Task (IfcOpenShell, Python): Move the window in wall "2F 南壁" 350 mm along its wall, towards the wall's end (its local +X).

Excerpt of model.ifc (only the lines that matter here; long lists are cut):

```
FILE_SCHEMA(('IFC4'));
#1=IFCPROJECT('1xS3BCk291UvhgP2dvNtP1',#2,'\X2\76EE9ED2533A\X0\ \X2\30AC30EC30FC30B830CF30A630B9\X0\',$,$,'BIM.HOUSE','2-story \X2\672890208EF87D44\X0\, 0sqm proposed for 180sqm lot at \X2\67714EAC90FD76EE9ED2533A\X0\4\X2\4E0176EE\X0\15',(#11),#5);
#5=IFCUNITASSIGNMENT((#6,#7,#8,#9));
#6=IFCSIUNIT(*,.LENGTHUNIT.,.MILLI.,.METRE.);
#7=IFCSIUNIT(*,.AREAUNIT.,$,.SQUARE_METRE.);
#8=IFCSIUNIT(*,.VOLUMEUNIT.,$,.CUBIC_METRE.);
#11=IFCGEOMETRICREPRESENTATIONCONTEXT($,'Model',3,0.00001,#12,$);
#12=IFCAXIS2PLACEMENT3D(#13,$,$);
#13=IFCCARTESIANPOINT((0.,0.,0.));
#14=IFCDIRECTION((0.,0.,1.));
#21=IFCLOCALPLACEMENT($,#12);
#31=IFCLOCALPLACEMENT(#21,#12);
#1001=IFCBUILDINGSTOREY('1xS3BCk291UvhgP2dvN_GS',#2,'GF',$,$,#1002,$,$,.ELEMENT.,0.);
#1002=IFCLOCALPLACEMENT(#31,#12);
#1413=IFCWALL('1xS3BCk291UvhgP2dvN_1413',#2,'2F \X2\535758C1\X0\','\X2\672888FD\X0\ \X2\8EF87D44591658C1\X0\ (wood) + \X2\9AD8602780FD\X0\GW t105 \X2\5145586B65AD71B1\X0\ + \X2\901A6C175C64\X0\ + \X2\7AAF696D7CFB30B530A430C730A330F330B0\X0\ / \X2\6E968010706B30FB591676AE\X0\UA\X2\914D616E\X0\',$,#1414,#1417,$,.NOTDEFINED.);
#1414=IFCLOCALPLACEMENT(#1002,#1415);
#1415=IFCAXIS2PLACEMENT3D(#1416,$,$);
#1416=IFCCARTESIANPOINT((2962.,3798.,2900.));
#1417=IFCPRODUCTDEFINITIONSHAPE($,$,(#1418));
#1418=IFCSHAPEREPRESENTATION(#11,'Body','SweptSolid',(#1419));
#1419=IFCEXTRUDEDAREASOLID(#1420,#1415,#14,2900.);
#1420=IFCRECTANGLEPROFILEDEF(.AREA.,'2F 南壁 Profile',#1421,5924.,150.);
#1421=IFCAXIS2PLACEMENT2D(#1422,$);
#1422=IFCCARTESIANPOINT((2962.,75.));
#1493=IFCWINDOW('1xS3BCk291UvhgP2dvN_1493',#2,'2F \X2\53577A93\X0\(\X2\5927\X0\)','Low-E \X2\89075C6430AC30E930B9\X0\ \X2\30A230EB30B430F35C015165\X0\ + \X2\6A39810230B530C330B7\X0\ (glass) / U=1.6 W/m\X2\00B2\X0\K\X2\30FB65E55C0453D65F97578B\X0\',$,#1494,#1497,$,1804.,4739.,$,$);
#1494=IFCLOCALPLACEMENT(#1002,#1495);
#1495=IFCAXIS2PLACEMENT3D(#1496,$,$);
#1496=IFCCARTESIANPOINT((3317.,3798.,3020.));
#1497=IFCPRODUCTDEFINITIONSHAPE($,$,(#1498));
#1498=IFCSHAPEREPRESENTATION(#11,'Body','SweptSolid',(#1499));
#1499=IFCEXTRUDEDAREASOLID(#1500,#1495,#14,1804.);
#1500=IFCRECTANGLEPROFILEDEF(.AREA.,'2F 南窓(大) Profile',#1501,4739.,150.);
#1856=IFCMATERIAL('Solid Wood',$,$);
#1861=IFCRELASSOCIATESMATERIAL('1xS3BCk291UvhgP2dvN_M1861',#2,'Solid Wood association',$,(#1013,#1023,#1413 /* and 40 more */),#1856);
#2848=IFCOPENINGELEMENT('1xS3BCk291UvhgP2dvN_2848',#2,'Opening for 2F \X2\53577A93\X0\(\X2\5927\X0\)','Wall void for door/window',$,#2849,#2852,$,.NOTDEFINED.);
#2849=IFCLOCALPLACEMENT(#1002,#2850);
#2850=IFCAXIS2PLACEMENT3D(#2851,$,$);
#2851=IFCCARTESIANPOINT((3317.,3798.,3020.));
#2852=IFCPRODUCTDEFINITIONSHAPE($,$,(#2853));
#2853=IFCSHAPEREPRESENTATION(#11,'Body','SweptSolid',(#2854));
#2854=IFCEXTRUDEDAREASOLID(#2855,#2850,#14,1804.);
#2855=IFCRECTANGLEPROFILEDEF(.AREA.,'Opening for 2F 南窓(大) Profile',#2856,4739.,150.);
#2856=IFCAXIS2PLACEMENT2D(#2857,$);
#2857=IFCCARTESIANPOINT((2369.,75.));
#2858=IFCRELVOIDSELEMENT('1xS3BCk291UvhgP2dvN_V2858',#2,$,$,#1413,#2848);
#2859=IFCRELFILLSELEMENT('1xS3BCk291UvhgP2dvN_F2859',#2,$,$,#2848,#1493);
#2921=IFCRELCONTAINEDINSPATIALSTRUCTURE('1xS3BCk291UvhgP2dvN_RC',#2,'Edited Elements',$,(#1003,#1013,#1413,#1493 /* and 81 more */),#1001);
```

```python
import ifcopenshell
import ifcopenshell.api.geometry
import ifcopenshell.util.placement
import ifcopenshell.util.unit

model = ifcopenshell.open("model.ifc")
unit_scale = ifcopenshell.util.unit.calculate_unit_scale(model)

window = model.by_guid("1xS3BCk291UvhgP2dvN_1493")
opening = window.FillsVoids[0].RelatingOpeningElement
wall = opening.VoidsElements[0].RelatingBuildingElement

wall_matrix = ifcopenshell.util.placement.get_local_placement(wall.ObjectPlacement)
shift = wall_matrix[:3, 0] * 0.35 / unit_scale
before = ifcopenshell.util.placement.get_local_placement(window.ObjectPlacement)[:3, 3].copy()

# The window is not placed relative to its opening, so move both.
for product in (opening, window):
    matrix = ifcopenshell.util.placement.get_local_placement(product.ObjectPlacement)
    matrix[:3, 3] += shift
    ifcopenshell.api.geometry.edit_object_placement(model, product=product, matrix=matrix, is_si=False)

after = ifcopenshell.util.placement.get_local_placement(window.ObjectPlacement)[:3, 3]
print("window moved by", (after - before).round(3) + 0.0)

model.write("model_edited.ifc")
```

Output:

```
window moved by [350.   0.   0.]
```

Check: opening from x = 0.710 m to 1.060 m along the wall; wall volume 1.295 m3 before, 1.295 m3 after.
